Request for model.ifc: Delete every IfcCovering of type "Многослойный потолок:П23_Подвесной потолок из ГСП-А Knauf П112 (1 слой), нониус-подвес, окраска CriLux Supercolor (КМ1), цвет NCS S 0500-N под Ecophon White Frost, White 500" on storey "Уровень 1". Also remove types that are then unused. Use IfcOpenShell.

First a look at what the model holds.

```python
import ifcopenshell
import ifcopenshell.util.element

model = ifcopenshell.open("model.ifc")
print(model.schema)
storey = next(s for s in model.by_type("IfcBuildingStorey") if s.Name == "Уровень 1")
coverings = [e for e in ifcopenshell.util.element.get_decomposition(storey) if e.is_a("IfcCovering")]
seen = {}
for e in coverings:
    element_type = ifcopenshell.util.element.get_type(e)
    name = element_type.Name if element_type not in (None, e) else None
    seen[name] = seen.get(name, 0) + 1
for name, count in sorted(seen.items(), key=str):
    print(count, "x", name)
```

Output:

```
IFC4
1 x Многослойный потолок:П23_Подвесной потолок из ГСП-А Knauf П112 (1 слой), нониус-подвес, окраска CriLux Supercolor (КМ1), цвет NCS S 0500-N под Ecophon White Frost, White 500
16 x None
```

```python
import ifcopenshell
import ifcopenshell.api.root
import ifcopenshell.util.element

model = ifcopenshell.open("model.ifc")

storey = next(s for s in model.by_type("IfcBuildingStorey") if s.Name == "Уровень 1")
coverings = [e for e in ifcopenshell.util.element.get_decomposition(storey) if e.is_a("IfcCovering")]
targets = [e for e in coverings if (t := ifcopenshell.util.element.get_type(e)) not in (None, e) and t.Name == "Многослойный потолок:П23_Подвесной потолок из ГСП-А Knauf П112 (1 слой), нониус-подвес, окраска CriLux Supercolor (КМ1), цвет NCS S 0500-N под Ecophon White Frost, White 500"]
types = {ifcopenshell.util.element.get_type(e) for e in targets} - {None, *targets}

for e in targets:
    ifcopenshell.api.root.remove_product(model, product=e)
print(len(targets), "removed")

unused = [t for t in types if not ifcopenshell.util.element.get_types(t)]
for t in unused:
    ifcopenshell.api.root.remove_product(model, product=t)
print(len(unused), "unused types removed")

model.write("model_v2.ifc")
```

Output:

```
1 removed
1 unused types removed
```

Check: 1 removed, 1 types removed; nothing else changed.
